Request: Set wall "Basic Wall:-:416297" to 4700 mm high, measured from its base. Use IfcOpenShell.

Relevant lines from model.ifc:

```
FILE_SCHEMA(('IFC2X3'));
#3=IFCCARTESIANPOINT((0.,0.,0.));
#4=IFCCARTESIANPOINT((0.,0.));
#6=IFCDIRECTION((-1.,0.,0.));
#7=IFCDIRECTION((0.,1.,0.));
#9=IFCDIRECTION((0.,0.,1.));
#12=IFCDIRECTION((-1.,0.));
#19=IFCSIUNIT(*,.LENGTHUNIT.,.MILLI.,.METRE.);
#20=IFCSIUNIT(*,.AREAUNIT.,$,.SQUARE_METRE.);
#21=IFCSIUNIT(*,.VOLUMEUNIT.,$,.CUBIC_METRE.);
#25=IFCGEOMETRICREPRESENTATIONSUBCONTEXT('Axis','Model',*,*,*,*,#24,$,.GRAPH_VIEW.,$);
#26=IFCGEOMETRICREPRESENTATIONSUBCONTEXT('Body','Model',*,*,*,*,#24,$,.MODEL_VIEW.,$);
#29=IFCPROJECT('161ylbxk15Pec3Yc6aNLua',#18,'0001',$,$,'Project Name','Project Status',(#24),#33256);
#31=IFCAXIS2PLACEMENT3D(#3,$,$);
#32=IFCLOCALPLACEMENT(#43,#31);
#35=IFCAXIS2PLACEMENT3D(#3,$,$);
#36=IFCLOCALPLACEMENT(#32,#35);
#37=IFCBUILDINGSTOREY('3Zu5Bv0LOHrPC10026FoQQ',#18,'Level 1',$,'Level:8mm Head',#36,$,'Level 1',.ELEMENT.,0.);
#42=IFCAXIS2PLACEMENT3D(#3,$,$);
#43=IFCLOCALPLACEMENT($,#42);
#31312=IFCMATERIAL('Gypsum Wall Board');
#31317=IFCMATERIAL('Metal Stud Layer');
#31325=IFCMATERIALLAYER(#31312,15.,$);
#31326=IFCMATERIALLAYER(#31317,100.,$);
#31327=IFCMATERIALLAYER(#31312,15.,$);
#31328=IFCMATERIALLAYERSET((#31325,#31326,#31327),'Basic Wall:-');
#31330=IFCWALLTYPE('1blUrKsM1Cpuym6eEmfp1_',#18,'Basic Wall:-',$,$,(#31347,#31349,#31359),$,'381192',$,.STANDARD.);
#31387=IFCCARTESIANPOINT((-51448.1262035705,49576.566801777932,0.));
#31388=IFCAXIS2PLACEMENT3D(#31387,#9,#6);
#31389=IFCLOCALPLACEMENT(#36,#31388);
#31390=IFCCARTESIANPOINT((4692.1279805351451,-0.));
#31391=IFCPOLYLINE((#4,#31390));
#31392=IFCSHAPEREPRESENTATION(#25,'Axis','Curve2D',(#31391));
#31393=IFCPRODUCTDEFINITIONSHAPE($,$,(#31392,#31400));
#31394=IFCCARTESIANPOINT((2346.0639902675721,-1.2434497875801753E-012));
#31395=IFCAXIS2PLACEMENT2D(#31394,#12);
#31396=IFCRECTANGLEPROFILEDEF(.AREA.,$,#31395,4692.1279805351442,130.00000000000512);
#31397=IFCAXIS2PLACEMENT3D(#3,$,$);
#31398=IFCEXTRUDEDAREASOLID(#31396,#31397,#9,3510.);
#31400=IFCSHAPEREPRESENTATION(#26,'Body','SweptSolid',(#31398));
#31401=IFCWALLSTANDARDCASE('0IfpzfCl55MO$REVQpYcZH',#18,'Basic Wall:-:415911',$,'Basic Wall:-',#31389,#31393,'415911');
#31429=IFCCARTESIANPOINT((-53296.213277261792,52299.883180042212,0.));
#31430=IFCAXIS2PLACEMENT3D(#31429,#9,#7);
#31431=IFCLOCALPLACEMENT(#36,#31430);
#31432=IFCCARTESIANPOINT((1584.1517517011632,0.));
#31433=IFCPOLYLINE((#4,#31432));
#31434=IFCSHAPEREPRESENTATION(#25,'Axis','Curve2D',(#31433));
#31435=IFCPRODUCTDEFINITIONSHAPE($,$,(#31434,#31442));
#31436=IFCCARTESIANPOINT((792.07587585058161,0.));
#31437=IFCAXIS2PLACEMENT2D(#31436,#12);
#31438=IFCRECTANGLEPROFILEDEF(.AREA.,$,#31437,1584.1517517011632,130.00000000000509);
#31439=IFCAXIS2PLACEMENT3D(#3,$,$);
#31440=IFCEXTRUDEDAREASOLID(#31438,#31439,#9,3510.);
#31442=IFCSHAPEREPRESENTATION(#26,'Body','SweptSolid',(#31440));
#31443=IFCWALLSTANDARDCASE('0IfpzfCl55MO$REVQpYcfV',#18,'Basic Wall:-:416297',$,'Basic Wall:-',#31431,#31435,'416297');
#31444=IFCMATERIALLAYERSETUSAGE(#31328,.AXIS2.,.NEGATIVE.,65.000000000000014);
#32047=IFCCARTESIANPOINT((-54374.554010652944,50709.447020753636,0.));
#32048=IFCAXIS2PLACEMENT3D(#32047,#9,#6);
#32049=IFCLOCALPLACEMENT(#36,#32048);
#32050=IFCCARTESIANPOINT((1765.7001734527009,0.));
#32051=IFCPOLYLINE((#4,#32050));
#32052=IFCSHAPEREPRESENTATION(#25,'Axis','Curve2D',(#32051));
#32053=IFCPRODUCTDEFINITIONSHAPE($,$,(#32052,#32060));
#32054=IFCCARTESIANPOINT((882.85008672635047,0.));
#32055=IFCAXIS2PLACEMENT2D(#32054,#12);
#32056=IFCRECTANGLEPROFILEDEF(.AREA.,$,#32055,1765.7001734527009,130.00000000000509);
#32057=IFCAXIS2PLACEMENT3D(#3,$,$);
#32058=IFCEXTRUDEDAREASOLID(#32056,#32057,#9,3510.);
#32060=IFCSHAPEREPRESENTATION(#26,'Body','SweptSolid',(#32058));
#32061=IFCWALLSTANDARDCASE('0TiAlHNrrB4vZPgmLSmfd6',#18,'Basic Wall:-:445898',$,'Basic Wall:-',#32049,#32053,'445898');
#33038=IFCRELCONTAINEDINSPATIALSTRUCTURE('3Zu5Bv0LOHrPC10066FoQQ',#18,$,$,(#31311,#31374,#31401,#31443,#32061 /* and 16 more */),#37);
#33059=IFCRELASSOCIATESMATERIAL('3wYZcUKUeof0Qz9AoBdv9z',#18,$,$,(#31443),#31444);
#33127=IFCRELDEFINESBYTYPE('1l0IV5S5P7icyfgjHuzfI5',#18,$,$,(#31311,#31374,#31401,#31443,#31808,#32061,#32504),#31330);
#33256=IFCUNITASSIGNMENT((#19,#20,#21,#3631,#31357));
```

```python
import ifcopenshell
import ifcopenshell.geom
import ifcopenshell.util.representation
import ifcopenshell.util.shape

model = ifcopenshell.open("model.ifc")
settings = ifcopenshell.geom.settings()


def volume(element):
    """Net volume in cubic metres, openings subtracted."""
    shape = ifcopenshell.geom.create_shape(settings, element)
    return ifcopenshell.util.shape.get_volume(shape.geometry)


wall = model.by_guid("0IfpzfCl55MO$REVQpYcfV")
before = volume(wall)

body = ifcopenshell.util.representation.get_representation(wall, "Model", "Body")
solid = body.Items[0]
old_height = solid.Depth
solid.Depth = 4700.0
after = volume(wall)

print(f"height {old_height:g} -> {solid.Depth:g}, volume {before:.3f} -> {after:.3f} m3")

model.write("model_rev.ifc")
```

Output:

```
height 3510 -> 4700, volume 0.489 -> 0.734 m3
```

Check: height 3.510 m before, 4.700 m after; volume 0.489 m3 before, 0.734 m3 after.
